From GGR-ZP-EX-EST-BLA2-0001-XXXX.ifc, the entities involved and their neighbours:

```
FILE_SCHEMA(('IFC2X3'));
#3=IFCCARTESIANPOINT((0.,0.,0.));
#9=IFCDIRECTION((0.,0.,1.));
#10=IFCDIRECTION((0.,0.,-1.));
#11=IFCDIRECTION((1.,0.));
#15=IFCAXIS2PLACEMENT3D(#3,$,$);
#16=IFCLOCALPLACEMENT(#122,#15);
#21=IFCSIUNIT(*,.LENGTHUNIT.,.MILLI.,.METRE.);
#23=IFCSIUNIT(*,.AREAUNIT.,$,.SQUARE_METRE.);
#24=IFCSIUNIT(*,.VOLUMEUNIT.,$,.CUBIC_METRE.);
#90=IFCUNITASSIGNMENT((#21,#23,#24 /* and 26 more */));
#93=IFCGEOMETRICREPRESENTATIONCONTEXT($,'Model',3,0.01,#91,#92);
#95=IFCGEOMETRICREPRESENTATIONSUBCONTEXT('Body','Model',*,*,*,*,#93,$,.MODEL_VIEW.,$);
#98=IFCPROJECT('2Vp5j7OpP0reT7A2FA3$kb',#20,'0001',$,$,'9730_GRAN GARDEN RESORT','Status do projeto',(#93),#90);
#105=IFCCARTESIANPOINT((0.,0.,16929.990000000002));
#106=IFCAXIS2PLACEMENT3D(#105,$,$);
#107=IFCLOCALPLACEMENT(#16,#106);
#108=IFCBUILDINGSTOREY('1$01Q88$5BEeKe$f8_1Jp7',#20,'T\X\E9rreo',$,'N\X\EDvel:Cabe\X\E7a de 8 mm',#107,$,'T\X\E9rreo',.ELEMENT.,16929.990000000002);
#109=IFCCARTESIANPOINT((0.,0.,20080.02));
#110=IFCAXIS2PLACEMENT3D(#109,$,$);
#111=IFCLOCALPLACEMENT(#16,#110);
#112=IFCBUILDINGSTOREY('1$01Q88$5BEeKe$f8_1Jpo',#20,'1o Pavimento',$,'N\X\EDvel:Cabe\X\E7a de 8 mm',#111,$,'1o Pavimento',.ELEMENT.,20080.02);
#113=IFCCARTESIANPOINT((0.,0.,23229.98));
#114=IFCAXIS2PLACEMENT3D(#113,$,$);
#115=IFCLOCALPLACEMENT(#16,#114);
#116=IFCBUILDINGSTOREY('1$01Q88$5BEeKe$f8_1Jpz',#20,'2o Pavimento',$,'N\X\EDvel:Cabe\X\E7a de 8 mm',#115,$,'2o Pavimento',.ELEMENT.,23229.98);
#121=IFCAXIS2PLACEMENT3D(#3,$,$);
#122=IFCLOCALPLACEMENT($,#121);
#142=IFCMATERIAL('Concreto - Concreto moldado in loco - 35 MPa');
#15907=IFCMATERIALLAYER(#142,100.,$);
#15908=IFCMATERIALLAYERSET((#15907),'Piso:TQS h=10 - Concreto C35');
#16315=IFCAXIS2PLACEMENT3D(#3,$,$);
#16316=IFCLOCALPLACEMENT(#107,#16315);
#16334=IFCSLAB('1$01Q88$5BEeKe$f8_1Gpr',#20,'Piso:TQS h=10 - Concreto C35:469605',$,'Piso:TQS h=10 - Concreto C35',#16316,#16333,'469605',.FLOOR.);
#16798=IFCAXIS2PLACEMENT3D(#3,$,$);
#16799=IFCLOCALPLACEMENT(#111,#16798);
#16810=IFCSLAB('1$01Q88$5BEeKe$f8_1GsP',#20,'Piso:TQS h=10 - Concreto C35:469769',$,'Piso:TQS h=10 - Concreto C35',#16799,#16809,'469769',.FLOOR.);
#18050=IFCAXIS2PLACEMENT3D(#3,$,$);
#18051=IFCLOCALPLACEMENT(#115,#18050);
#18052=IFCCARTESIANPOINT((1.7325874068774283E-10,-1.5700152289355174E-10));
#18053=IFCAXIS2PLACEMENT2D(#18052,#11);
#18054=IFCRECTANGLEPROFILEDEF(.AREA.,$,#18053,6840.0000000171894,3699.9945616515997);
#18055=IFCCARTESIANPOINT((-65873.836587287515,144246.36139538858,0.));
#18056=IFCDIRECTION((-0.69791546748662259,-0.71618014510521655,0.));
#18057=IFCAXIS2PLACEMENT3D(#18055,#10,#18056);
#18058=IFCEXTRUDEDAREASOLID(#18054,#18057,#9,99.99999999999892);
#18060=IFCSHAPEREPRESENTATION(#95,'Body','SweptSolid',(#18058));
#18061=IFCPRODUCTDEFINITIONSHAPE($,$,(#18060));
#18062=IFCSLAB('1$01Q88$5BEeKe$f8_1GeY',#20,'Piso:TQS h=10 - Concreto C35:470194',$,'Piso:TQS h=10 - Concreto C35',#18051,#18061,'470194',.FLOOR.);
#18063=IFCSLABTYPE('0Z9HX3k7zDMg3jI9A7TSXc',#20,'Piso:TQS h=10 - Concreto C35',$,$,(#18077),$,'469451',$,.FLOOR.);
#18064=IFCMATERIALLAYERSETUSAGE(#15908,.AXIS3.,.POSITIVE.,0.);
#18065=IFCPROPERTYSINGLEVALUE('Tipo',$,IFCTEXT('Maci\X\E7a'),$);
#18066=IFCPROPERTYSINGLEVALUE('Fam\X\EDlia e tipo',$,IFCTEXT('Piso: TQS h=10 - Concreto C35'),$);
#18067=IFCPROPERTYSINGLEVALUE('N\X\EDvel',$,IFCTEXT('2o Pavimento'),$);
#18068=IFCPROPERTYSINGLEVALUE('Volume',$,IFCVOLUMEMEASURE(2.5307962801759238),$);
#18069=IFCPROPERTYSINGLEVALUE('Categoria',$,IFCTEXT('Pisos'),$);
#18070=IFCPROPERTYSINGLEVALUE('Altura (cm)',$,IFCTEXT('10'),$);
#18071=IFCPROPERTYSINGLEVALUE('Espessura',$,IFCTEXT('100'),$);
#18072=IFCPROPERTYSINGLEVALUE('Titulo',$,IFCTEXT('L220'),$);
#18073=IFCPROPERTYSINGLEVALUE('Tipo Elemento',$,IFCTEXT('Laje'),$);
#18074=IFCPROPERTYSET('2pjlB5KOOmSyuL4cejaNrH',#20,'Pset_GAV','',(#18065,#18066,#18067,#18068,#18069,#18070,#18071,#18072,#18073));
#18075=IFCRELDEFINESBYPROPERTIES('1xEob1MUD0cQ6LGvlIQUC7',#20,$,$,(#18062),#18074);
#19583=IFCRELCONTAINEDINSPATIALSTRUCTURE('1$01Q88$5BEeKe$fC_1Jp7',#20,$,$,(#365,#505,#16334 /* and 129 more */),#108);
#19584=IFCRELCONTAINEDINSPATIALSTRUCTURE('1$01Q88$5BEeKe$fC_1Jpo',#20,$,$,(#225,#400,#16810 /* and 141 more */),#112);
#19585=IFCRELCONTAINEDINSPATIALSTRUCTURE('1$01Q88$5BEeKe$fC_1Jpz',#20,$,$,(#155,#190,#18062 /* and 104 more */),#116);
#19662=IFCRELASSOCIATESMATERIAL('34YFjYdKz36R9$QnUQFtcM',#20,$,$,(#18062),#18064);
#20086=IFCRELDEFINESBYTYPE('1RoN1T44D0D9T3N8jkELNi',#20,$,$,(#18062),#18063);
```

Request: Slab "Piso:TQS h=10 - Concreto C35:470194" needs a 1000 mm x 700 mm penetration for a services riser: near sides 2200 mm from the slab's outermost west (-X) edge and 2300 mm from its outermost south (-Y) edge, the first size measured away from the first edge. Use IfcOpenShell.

```python
import numpy as np
import ifcopenshell
import ifcopenshell.api.feature
import ifcopenshell.api.geometry
import ifcopenshell.api.pset
import ifcopenshell.api.root
import ifcopenshell.geom
import ifcopenshell.util.element
import ifcopenshell.util.placement
import ifcopenshell.util.representation
import ifcopenshell.util.shape
import ifcopenshell.util.unit

model = ifcopenshell.open("GGR-ZP-EX-EST-BLA2-0001-XXXX.ifc")
unit_scale = ifcopenshell.util.unit.calculate_unit_scale(model)
volume_scale = ifcopenshell.util.unit.calculate_unit_scale(model, "VOLUMEUNIT")
settings = ifcopenshell.geom.settings()


def volume(element):
    """Net volume in cubic metres, openings subtracted."""
    shape = ifcopenshell.geom.create_shape(settings, element)
    return ifcopenshell.util.shape.get_volume(shape.geometry)


slab = model.by_guid("1$01Q88$5BEeKe$f8_1GeY")
before = volume(slab)

# Extent in the slab's own axes, in metres. The edges named are its -X and -Y sides.
slab_shape = ifcopenshell.geom.create_shape(settings, slab)
vertices = ifcopenshell.util.shape.get_vertices(slab_shape.geometry)
x_min, y_min, bottom = vertices.min(axis=0)
top = vertices[:, 2].max()

opening = ifcopenshell.api.root.create_entity(model, ifc_class="IfcOpeningElement", name="Services riser opening")
context = ifcopenshell.util.representation.get_context(model, "Model", "Body", "MODEL_VIEW")
width, depth = 1, 0.7
outline = [(0.0, 0.0), (width, 0.0), (width, depth), (0.0, depth), (0.0, 0.0)]
# Overshoot both faces by 50 mm so the cut is clean.
shape = ifcopenshell.api.geometry.add_slab_representation(
    model, context=context, depth=top - bottom + 0.1, polyline=outline
)
ifcopenshell.api.geometry.assign_representation(model, product=opening, representation=shape)

matrix = ifcopenshell.util.placement.get_local_placement(slab.ObjectPlacement)
matrix[:, 3] = matrix @ np.append(np.array([x_min + 2.2, y_min + 2.3, bottom - 0.05]) / unit_scale, 1.0)
ifcopenshell.api.geometry.edit_object_placement(model, product=opening, matrix=matrix, is_si=False)
ifcopenshell.api.feature.add_feature(model, feature=opening, element=slab)

after = volume(slab)

# Update the slab's stored quantities.
pset = model.by_id(ifcopenshell.util.element.get_pset(slab, "Pset_GAV", should_inherit=False)["id"])
ifcopenshell.api.pset.edit_pset(model, pset=pset, properties={
    "Volume": model.create_entity("IfcVolumeMeasure", after / volume_scale),
})

print(f"slab volume {before:.3f} -> {after:.3f} m3")

model.write("GGR-ZP-EX-EST-BLA2-0001-XXXX_v2.ifc")
```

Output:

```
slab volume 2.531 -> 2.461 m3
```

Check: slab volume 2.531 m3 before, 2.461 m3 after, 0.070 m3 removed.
